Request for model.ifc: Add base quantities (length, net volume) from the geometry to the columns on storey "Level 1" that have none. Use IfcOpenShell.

First a look at what the model holds.

```python
import ifcopenshell
import ifcopenshell.util.element
import ifcopenshell.util.unit

model = ifcopenshell.open("model.ifc")
print(model.schema)
for unit_type in ("LENGTHUNIT", "AREAUNIT", "VOLUMEUNIT"):
    print(unit_type, ifcopenshell.util.unit.calculate_unit_scale(model, unit_type))
storey = next(s for s in model.by_type("IfcBuildingStorey") if s.Name == "Level 1")
columns = [e for e in ifcopenshell.util.element.get_decomposition(storey) if e.is_a("IfcColumn")]
for e in sorted(columns, key=lambda e: e.id()):
    print(e.id(), e.is_a(), e.Name, list(ifcopenshell.util.element.get_psets(e, qtos_only=True)), sep=" | ")
```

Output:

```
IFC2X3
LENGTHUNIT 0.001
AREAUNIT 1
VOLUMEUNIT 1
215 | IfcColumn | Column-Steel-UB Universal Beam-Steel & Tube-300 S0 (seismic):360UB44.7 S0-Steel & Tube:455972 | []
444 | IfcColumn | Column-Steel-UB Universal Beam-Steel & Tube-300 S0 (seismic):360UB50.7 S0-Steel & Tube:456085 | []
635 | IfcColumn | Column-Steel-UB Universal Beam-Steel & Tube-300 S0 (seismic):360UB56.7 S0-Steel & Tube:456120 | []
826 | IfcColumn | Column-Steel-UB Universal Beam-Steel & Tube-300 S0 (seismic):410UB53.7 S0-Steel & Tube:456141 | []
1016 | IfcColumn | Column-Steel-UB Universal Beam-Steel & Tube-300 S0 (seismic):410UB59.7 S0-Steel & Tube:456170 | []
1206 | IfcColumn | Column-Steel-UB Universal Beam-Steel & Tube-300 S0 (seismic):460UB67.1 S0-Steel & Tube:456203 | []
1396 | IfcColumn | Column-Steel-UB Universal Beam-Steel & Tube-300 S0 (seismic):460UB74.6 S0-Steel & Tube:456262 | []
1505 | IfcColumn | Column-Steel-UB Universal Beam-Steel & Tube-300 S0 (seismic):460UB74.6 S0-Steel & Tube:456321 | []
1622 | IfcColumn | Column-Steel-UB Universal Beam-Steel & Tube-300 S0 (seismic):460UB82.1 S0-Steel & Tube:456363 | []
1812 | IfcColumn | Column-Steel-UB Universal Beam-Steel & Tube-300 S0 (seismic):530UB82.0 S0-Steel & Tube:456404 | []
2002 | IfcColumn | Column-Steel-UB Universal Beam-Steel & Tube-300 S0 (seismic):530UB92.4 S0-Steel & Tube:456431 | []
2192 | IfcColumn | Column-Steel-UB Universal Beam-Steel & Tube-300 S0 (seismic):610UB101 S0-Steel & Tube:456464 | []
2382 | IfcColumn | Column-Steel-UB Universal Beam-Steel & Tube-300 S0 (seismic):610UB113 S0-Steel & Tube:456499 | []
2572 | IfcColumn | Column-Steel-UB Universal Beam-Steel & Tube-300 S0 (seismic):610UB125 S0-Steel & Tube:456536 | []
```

```python
import ifcopenshell
import ifcopenshell.api.pset
import ifcopenshell.geom
import ifcopenshell.util.element
import ifcopenshell.util.shape
import ifcopenshell.util.unit

model = ifcopenshell.open("model.ifc")
unit_scale = ifcopenshell.util.unit.calculate_unit_scale(model)
volume_scale = ifcopenshell.util.unit.calculate_unit_scale(model, "VOLUMEUNIT")
settings = ifcopenshell.geom.settings()

storey = next(s for s in model.by_type("IfcBuildingStorey") if s.Name == "Level 1")
columns = [e for e in ifcopenshell.util.element.get_decomposition(storey) if e.is_a("IfcColumn")]

for e in sorted(columns, key=lambda e: e.id()):
    if ifcopenshell.util.element.get_psets(e, qtos_only=True, should_inherit=False):
        continue
    # Geometry comes back in metres, in the element's own axes.
    shape = ifcopenshell.geom.create_shape(settings, e)
    values = {
        "Length": ifcopenshell.util.shape.get_z(shape.geometry) / unit_scale,
        "NetVolume": ifcopenshell.util.shape.get_volume(shape.geometry) / volume_scale,
    }
    qto = ifcopenshell.api.pset.add_qto(model, product=e, name="BaseQuantities")
    ifcopenshell.api.pset.edit_qto(model, qto=qto, properties=values)
    print(e.id(), {k: round(v, 3) for k, v in values.items()})

model.write("model_updated.ifc")
```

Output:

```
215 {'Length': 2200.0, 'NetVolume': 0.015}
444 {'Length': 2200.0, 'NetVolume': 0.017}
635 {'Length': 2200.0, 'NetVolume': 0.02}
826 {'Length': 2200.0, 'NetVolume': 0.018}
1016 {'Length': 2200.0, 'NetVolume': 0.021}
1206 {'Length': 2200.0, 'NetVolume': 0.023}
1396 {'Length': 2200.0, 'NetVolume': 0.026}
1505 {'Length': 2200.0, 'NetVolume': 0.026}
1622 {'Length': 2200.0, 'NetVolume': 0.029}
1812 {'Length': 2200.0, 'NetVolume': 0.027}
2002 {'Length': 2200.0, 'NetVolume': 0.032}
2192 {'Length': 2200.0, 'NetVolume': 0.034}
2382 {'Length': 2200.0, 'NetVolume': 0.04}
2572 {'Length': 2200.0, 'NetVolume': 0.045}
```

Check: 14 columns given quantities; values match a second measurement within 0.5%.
